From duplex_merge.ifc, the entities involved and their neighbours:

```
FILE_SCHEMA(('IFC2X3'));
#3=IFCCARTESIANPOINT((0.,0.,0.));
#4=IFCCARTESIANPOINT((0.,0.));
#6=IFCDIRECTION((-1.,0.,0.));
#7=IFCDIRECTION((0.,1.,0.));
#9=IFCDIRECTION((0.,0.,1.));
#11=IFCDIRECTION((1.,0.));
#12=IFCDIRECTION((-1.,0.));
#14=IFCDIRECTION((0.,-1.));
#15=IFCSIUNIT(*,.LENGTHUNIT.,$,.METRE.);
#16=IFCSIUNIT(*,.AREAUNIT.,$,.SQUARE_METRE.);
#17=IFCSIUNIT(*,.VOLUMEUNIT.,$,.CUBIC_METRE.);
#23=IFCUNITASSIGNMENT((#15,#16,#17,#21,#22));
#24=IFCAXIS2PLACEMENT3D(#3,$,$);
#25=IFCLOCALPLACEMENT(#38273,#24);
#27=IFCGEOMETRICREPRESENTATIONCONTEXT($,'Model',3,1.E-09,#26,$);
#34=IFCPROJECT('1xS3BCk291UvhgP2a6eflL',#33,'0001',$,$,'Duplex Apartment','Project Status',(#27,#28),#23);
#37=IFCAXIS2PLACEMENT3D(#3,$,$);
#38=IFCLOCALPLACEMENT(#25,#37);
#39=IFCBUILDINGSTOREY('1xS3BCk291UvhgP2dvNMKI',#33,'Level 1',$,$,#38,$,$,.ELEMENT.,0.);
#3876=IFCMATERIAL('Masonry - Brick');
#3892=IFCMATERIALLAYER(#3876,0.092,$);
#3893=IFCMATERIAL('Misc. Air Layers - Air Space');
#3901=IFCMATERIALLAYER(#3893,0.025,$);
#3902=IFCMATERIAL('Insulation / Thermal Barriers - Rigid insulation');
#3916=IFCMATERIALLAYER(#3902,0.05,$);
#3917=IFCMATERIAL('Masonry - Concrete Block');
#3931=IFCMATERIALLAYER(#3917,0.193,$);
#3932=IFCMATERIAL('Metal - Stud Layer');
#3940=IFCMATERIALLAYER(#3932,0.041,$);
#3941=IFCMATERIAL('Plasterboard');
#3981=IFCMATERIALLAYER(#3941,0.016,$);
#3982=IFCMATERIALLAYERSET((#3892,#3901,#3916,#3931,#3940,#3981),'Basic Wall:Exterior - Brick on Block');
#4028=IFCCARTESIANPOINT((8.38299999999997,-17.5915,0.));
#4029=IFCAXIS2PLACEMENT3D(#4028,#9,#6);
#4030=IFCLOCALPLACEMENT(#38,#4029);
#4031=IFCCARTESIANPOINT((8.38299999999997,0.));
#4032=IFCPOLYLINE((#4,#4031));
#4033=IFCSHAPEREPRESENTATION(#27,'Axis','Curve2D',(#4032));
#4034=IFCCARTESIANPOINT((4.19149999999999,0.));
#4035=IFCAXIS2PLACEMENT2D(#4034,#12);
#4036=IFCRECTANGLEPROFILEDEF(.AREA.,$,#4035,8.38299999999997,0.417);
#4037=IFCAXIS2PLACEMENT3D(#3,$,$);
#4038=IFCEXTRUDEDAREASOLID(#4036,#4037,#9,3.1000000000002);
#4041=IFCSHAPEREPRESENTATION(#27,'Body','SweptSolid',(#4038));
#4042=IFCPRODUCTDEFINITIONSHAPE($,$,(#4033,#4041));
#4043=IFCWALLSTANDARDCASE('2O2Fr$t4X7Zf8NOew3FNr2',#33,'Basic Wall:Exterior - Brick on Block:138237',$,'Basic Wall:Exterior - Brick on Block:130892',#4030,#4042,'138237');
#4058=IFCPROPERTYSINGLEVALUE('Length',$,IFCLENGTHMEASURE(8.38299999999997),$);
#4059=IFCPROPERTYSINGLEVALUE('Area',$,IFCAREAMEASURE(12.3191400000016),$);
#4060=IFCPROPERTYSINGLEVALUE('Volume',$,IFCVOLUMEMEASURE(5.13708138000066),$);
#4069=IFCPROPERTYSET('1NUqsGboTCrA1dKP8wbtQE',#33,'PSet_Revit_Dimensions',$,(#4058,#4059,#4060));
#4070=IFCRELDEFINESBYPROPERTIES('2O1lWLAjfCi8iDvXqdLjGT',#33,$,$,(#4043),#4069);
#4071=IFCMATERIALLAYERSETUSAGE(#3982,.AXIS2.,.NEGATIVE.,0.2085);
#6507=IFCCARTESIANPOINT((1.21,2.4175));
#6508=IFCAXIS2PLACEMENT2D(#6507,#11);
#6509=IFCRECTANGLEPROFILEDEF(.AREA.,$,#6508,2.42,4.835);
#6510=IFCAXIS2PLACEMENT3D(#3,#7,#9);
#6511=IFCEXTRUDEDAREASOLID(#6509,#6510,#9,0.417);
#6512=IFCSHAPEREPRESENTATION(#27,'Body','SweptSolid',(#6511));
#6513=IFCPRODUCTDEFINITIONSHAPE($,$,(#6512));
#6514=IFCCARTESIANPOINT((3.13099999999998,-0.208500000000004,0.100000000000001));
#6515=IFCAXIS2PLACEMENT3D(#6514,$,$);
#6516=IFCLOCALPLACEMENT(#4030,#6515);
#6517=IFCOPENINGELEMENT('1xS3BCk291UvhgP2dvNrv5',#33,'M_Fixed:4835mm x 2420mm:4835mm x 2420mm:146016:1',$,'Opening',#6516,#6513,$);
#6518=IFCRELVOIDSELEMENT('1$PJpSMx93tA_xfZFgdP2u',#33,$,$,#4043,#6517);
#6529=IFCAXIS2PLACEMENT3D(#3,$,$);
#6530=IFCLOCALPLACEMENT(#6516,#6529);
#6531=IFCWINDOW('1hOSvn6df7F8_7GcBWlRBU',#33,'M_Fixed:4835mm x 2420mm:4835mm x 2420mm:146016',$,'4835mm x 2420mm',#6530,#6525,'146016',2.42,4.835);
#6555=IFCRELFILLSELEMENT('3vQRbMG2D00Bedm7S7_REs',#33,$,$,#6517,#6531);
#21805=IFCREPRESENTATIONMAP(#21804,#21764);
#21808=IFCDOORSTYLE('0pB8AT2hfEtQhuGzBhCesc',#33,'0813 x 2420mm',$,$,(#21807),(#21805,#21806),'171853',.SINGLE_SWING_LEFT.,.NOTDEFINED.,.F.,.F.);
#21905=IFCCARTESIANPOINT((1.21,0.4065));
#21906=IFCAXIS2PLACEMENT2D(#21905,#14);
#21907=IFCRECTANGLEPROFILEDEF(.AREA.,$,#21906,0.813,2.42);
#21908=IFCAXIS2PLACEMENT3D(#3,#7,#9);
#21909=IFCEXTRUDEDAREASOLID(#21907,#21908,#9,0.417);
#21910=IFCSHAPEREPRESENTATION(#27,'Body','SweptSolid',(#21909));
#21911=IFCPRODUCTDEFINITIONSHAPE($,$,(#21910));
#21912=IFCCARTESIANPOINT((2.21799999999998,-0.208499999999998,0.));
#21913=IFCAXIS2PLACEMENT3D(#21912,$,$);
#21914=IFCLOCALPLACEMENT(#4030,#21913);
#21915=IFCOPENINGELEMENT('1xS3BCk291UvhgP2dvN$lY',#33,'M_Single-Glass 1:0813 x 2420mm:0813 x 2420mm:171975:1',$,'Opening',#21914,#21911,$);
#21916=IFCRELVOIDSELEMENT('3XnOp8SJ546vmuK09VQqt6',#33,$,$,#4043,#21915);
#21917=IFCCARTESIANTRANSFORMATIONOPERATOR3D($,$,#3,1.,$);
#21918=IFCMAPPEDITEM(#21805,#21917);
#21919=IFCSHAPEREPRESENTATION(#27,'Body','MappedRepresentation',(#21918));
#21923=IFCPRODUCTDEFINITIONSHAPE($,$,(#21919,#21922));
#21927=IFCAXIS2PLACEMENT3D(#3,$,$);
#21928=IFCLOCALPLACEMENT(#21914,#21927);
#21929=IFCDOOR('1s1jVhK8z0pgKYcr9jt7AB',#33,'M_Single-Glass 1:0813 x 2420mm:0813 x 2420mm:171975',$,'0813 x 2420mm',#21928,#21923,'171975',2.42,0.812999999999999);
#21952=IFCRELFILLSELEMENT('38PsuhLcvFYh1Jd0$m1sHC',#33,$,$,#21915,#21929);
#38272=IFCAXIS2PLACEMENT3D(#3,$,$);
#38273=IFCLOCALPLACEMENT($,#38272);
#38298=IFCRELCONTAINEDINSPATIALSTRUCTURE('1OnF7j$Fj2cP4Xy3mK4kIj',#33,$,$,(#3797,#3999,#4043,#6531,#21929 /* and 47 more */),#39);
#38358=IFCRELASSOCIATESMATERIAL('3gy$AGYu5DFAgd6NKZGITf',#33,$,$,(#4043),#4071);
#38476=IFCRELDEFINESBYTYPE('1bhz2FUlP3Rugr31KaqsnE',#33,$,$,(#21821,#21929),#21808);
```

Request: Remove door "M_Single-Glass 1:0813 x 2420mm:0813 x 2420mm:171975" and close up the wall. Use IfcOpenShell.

```python
import ifcopenshell
import ifcopenshell.api.feature
import ifcopenshell.api.pset
import ifcopenshell.api.root
import ifcopenshell.geom
import ifcopenshell.util.element
import ifcopenshell.util.shape
import ifcopenshell.util.unit

model = ifcopenshell.open("duplex_merge.ifc")
area_scale = ifcopenshell.util.unit.calculate_unit_scale(model, "AREAUNIT")
volume_scale = ifcopenshell.util.unit.calculate_unit_scale(model, "VOLUMEUNIT")
settings = ifcopenshell.geom.settings()


def volume(element):
    """Net volume in cubic metres, openings subtracted."""
    shape = ifcopenshell.geom.create_shape(settings, element)
    return ifcopenshell.util.shape.get_volume(shape.geometry)


door = model.by_guid("1s1jVhK8z0pgKYcr9jt7AB")
opening = door.FillsVoids[0].RelatingOpeningElement
wall = opening.VoidsElements[0].RelatingBuildingElement
before = volume(wall)

ifcopenshell.api.root.remove_product(model, product=door)
ifcopenshell.api.feature.remove_feature(model, feature=opening)

after = volume(wall)
thickness = 0.417  # wall thickness in metres

# Update the wall's stored quantities.
pset = model.by_id(ifcopenshell.util.element.get_pset(wall, "PSet_Revit_Dimensions", should_inherit=False)["id"])
ifcopenshell.api.pset.edit_pset(model, pset=pset, properties={
    "Area": model.create_entity("IfcAreaMeasure", after / thickness / area_scale),
    "Volume": model.create_entity("IfcVolumeMeasure", after / volume_scale),
})

print(f"wall volume {before:.3f} -> {after:.3f} m3")

model.write("duplex_merge_updated.ifc")
```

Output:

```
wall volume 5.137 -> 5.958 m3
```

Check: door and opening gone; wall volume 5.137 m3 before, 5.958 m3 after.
